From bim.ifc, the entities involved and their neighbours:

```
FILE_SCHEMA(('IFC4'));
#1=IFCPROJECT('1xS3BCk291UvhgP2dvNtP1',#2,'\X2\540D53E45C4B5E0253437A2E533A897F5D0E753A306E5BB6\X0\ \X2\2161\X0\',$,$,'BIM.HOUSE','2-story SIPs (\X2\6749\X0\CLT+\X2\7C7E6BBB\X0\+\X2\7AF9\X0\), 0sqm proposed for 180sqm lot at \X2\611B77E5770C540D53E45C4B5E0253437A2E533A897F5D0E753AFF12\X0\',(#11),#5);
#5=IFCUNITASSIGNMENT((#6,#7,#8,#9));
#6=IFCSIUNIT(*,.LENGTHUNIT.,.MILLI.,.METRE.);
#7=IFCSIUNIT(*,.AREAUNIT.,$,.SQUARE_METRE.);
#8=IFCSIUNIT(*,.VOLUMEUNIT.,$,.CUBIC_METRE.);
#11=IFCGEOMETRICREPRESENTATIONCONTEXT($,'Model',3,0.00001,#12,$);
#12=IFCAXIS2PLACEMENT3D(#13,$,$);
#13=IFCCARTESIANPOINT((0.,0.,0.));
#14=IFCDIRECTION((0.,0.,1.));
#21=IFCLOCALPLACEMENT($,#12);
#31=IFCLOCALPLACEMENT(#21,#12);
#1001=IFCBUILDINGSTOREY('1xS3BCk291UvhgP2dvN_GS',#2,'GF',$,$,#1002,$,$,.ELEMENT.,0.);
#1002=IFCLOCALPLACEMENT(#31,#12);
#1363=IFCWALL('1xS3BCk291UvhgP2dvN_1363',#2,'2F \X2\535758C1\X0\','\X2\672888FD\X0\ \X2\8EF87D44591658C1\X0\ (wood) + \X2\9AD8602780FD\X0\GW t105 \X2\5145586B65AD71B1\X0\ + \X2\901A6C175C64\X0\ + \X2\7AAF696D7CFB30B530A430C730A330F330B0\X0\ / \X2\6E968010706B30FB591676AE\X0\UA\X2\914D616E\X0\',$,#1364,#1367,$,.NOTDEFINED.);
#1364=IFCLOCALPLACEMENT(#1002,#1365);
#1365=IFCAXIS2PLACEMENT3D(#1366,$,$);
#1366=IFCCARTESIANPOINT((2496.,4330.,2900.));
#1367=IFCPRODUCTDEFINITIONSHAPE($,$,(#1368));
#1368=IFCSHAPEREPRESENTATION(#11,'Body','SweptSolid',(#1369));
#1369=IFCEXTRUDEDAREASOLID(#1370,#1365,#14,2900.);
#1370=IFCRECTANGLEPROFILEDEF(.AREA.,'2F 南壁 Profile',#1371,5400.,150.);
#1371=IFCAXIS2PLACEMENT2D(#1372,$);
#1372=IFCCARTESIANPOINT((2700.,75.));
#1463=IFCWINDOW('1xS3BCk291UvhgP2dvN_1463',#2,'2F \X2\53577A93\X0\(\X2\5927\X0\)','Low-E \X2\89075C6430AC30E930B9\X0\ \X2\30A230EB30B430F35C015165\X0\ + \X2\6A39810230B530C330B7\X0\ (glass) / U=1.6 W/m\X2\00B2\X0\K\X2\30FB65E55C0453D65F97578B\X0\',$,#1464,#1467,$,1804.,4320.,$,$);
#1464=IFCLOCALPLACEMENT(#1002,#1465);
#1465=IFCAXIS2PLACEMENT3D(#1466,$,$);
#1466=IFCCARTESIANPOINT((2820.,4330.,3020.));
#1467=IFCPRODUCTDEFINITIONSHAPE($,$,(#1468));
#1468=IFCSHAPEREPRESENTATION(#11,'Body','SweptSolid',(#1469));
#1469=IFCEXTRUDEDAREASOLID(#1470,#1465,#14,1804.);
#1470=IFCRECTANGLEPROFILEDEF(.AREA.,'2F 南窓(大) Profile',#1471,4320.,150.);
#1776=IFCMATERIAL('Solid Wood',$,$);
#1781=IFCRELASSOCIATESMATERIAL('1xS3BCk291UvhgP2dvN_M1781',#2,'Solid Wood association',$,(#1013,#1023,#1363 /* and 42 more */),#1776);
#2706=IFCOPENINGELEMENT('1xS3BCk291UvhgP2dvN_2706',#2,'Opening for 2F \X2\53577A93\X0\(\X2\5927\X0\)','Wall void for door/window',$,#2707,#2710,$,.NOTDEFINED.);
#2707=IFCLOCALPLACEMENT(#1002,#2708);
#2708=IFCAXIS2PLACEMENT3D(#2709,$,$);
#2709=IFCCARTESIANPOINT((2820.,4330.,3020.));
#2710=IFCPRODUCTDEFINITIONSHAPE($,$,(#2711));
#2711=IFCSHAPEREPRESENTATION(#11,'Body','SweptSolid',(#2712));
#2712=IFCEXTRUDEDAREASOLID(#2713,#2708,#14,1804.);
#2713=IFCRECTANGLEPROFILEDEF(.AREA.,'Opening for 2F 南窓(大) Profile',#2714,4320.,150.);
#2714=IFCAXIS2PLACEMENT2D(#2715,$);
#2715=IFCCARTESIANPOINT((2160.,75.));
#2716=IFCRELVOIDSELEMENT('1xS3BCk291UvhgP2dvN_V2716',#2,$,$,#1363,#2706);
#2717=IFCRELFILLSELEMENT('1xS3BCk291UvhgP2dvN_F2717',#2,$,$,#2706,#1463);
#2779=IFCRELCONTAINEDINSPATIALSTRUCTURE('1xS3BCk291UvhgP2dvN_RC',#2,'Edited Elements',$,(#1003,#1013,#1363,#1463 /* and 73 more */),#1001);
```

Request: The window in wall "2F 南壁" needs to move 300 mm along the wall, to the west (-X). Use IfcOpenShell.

```python
import ifcopenshell
import ifcopenshell.api.geometry
import ifcopenshell.util.placement
import ifcopenshell.util.unit

model = ifcopenshell.open("bim.ifc")
unit_scale = ifcopenshell.util.unit.calculate_unit_scale(model)

window = model.by_guid("1xS3BCk291UvhgP2dvN_1463")
opening = window.FillsVoids[0].RelatingOpeningElement
wall = opening.VoidsElements[0].RelatingBuildingElement

wall_matrix = ifcopenshell.util.placement.get_local_placement(wall.ObjectPlacement)
shift = wall_matrix[:3, 0] * -0.3 / unit_scale
before = ifcopenshell.util.placement.get_local_placement(window.ObjectPlacement)[:3, 3].copy()

# The window is not placed relative to its opening, so move both.
for product in (opening, window):
    matrix = ifcopenshell.util.placement.get_local_placement(product.ObjectPlacement)
    matrix[:3, 3] += shift
    ifcopenshell.api.geometry.edit_object_placement(model, product=product, matrix=matrix, is_si=False)

after = ifcopenshell.util.placement.get_local_placement(window.ObjectPlacement)[:3, 3]
print("window moved by", (after - before).round(3) + 0.0)

model.write("bim_rev.ifc")
```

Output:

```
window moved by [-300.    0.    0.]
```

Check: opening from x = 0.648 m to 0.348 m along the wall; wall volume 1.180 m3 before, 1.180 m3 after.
